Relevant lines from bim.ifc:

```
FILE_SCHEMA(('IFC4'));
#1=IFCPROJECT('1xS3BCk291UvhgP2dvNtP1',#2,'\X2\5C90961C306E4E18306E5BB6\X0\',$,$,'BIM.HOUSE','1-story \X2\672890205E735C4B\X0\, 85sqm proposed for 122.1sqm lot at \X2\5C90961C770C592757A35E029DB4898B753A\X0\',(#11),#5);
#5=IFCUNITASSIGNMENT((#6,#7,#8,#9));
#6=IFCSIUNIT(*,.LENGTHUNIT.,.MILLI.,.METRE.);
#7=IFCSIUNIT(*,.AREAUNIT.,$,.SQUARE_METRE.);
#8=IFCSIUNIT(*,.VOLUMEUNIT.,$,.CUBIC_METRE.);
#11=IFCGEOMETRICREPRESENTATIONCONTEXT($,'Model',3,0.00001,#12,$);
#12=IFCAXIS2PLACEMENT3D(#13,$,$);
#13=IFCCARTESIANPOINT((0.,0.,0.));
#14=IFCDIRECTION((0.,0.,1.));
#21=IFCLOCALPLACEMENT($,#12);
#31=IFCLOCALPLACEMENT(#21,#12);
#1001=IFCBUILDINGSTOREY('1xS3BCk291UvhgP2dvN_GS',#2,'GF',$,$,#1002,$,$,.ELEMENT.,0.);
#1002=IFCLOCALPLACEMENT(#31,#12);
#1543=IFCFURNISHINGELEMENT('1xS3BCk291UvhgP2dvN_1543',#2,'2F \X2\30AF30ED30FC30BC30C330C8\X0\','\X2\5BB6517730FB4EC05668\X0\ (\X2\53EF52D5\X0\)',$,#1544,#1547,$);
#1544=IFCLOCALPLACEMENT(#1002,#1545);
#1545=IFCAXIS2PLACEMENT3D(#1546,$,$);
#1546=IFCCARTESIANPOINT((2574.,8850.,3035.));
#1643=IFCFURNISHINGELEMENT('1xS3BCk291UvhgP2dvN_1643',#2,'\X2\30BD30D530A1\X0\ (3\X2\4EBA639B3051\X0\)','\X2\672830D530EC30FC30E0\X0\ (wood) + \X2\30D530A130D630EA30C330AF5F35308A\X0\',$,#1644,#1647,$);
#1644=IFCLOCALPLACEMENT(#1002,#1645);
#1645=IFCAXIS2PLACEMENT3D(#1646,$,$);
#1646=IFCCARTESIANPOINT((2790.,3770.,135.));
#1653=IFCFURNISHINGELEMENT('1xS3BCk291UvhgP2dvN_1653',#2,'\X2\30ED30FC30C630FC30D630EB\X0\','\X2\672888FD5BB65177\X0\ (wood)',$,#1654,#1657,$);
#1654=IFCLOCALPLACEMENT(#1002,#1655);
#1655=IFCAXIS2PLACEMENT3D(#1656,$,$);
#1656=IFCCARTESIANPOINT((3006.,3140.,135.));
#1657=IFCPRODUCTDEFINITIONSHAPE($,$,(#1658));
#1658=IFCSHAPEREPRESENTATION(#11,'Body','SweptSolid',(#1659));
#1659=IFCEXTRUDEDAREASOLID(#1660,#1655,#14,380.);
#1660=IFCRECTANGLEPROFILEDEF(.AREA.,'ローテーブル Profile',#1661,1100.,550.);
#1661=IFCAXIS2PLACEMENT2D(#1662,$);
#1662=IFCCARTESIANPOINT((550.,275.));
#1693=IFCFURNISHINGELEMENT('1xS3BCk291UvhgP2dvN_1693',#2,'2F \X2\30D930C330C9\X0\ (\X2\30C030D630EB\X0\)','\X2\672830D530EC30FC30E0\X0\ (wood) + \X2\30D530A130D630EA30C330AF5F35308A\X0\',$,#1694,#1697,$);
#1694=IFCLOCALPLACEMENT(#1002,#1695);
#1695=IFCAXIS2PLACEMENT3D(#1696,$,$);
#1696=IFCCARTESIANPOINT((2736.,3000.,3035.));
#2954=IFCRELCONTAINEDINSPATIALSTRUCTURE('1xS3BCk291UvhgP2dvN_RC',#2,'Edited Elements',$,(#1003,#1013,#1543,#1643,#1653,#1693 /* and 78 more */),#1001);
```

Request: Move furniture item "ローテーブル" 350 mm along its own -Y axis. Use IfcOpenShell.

```python
import ifcopenshell
import ifcopenshell.api.geometry
import ifcopenshell.util.placement

model = ifcopenshell.open("bim.ifc")

item = model.by_guid("1xS3BCk291UvhgP2dvN_1653")
matrix = ifcopenshell.util.placement.get_local_placement(item.ObjectPlacement)
matrix[:3, 3] -= matrix[:3, 1] * 350.0
ifcopenshell.api.geometry.edit_object_placement(model, product=item, matrix=matrix, is_si=False)

print(ifcopenshell.util.placement.get_local_placement(item.ObjectPlacement).round(3) + 0.0)

model.write("bim_edited.ifc")
```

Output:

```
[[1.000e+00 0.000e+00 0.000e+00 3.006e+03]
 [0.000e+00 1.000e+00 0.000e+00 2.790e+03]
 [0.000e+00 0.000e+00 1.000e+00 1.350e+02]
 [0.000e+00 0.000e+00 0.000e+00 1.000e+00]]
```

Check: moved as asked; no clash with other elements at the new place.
